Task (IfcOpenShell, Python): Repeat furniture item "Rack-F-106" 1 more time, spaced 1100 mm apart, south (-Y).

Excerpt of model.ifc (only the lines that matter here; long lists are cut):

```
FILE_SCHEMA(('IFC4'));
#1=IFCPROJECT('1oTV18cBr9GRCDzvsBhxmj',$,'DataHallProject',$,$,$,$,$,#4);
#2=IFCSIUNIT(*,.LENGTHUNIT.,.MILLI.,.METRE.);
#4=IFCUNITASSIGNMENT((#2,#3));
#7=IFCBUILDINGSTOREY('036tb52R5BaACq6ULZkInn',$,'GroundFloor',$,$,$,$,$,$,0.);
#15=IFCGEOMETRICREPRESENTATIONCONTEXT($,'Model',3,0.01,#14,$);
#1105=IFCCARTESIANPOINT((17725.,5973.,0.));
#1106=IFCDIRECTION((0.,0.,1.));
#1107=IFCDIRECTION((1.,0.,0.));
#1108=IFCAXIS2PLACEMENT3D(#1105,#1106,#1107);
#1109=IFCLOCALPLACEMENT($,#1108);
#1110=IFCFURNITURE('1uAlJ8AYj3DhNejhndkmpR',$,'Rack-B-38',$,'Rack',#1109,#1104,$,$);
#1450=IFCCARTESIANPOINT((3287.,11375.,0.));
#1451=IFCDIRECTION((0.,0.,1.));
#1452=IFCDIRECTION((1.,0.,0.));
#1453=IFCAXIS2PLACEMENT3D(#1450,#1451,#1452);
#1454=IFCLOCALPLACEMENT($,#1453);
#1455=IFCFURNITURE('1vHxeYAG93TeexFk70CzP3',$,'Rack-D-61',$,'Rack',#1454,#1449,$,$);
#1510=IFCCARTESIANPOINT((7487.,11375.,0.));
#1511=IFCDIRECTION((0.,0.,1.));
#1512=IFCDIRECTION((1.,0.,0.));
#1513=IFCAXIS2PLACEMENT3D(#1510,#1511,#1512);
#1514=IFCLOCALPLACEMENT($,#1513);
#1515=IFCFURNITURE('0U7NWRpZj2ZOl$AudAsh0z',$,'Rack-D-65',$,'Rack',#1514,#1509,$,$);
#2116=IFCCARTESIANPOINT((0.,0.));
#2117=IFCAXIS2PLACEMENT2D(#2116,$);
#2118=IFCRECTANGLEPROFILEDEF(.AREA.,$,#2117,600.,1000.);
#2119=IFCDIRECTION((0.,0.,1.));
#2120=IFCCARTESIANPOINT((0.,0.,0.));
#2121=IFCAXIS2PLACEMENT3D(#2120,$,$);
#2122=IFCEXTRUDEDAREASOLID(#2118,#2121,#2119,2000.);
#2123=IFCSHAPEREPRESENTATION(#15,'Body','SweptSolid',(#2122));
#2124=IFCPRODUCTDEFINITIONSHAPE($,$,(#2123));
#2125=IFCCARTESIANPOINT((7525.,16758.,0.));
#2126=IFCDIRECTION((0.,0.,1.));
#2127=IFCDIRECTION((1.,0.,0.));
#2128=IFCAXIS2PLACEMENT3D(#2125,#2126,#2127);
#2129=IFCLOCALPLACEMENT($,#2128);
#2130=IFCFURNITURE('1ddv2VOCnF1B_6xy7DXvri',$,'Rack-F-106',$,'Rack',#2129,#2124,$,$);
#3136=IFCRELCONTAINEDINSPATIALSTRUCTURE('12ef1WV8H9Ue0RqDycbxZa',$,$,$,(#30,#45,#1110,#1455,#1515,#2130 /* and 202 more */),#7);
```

```python
import numpy as np
import ifcopenshell
import ifcopenshell.api.geometry
import ifcopenshell.api.root
import ifcopenshell.util.element
import ifcopenshell.util.placement

model = ifcopenshell.open("model.ifc")

source = model.by_guid("1ddv2VOCnF1B_6xy7DXvri")
base = ifcopenshell.util.placement.get_local_placement(source.ObjectPlacement)
step = np.array([0.0, -1.0, 0.0]) * 1100.0

for i in range(1, 2):
    copy = ifcopenshell.api.root.copy_class(model, product=source)
    copy.Representation = ifcopenshell.util.element.copy_deep(
        model, source.Representation, exclude=["IfcGeometricRepresentationContext", "IfcRepresentationMap"]
    )
    matrix = base.copy()
    matrix[:3, 3] += i * step
    print("added at", matrix[:3, 3].round(3) + 0.0)
    ifcopenshell.api.geometry.edit_object_placement(model, product=copy, matrix=matrix, is_si=False)

model.write("model-out.ifc")
```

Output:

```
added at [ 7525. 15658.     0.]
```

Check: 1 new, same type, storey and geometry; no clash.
